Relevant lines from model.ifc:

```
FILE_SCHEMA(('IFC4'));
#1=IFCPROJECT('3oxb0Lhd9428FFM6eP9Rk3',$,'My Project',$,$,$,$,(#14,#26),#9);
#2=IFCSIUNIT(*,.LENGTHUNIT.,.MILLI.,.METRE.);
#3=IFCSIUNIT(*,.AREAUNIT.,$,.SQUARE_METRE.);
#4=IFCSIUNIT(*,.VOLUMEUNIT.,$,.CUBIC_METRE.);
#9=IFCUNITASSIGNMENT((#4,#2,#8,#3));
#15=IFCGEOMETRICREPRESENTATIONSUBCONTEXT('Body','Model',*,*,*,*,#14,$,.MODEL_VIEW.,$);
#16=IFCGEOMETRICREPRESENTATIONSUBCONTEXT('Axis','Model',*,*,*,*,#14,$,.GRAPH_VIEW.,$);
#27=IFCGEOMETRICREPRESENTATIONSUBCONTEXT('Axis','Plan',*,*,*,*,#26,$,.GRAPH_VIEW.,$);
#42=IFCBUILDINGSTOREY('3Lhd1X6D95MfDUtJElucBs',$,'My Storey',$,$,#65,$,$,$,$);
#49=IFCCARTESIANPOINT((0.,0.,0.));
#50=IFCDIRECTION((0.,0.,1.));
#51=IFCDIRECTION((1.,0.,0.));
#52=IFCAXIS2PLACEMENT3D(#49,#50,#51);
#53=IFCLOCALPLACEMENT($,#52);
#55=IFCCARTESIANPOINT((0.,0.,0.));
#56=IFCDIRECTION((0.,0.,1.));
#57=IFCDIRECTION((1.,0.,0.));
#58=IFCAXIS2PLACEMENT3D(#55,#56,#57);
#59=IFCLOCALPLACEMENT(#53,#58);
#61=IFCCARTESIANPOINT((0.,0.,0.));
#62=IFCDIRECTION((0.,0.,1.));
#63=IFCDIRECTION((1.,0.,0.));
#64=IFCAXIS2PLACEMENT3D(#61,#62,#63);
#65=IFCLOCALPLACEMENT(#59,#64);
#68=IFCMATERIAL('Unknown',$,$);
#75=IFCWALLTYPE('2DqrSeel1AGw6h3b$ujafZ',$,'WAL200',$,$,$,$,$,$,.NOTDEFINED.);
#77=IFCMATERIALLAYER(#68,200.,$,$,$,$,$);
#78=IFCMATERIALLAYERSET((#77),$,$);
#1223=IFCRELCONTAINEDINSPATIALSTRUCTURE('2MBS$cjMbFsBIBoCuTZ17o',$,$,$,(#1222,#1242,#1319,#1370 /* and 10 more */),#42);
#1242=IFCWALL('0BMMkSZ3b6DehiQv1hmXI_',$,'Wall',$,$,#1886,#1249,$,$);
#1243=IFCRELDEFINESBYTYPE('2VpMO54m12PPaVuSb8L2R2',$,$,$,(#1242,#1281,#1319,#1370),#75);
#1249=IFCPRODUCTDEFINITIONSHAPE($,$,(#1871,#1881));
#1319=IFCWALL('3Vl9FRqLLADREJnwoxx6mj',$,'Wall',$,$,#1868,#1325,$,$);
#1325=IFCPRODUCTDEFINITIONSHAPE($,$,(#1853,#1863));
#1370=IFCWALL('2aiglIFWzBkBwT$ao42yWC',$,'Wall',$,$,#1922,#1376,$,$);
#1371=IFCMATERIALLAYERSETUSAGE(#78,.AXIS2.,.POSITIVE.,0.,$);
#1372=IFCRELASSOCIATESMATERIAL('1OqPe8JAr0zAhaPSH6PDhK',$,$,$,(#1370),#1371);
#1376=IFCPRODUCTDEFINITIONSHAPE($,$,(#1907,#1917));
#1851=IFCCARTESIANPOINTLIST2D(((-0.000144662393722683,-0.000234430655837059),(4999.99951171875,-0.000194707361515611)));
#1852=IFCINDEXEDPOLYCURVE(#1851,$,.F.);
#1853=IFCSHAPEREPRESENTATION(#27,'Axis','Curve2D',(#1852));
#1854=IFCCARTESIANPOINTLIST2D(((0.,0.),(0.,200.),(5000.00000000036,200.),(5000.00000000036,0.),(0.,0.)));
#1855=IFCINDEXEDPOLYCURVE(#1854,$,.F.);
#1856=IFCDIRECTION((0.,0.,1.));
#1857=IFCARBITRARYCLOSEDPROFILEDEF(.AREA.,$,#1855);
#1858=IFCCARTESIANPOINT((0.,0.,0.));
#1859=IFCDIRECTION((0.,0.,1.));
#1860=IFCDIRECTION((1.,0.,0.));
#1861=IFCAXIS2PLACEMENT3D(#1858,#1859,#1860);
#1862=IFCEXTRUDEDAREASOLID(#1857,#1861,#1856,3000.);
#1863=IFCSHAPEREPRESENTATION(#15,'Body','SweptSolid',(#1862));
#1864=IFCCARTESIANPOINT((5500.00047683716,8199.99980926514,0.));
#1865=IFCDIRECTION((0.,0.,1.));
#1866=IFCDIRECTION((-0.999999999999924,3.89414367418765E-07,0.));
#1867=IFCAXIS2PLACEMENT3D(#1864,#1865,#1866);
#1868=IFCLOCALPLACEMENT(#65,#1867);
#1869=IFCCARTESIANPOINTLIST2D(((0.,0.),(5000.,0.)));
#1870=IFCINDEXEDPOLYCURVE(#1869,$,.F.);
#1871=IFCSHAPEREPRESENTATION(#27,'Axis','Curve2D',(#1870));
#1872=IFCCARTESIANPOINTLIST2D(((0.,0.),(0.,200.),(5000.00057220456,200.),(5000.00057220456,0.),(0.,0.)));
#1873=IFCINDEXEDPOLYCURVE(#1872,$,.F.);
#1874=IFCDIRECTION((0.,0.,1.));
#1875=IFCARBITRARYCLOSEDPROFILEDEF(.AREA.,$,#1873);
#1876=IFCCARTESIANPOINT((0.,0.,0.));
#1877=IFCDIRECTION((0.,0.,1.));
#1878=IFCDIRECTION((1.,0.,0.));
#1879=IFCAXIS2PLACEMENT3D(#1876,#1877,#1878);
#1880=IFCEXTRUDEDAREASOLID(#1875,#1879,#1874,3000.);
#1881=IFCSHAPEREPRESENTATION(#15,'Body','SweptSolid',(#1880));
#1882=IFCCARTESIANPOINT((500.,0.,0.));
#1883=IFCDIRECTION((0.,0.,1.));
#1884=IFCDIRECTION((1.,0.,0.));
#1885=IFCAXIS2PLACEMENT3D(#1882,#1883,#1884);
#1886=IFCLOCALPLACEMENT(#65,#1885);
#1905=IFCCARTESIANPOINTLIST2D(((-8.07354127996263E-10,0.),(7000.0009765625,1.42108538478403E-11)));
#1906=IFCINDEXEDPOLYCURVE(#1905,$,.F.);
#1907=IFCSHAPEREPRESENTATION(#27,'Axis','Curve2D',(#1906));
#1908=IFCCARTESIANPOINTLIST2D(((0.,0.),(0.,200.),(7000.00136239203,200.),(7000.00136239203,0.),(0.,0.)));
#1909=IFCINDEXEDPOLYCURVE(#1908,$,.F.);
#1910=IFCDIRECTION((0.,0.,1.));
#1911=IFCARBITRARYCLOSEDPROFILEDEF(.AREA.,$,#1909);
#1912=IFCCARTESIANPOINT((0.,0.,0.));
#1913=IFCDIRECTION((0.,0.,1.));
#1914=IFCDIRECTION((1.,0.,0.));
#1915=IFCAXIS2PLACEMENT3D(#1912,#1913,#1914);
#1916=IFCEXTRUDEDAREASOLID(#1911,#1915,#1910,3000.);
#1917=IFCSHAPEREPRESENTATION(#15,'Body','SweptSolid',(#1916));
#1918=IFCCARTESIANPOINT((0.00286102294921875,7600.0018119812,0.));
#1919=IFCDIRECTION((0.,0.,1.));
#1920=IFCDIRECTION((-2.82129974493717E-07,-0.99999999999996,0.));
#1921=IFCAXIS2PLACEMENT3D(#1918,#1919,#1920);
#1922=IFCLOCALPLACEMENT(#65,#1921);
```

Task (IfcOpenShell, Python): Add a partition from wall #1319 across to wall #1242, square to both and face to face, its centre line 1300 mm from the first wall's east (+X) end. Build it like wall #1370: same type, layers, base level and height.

```python
import numpy as np
import ifcopenshell
import ifcopenshell.api.geometry
import ifcopenshell.api.material
import ifcopenshell.api.pset
import ifcopenshell.api.root
import ifcopenshell.api.spatial
import ifcopenshell.api.type
import ifcopenshell.geom
import ifcopenshell.util.element
import ifcopenshell.util.placement
import ifcopenshell.util.representation
import ifcopenshell.util.shape
import ifcopenshell.util.unit

model = ifcopenshell.open("model.ifc")
unit_scale = ifcopenshell.util.unit.calculate_unit_scale(model)
settings = ifcopenshell.geom.settings()
settings.set("use-world-coords", True)

start_wall = model.by_id(1319)
end_wall = model.by_guid("0BMMkSZ3b6DehiQv1hmXI_")
like = model.by_id(1370)
matrix = ifcopenshell.util.placement.get_local_placement(start_wall.ObjectPlacement)
matrix[:3, 3] *= unit_scale


def extent(element):
    """Bounding box in the first wall's axes, in metres."""
    shape = ifcopenshell.geom.create_shape(settings, element)
    points = (ifcopenshell.util.shape.get_vertices(shape.geometry) - matrix[:3, 3]) @ matrix[:3, :3]
    return points.min(axis=0), points.max(axis=0)


y_start = extent(start_wall)[1][1]
y_end = extent(end_wall)[0][1]
like_min, like_max = extent(like)
length, height = float(abs(y_end - y_start)), float(like_max[2] - like_min[2])
layer_set = ifcopenshell.util.element.get_material(like, should_skip_usage=True)
thickness = sum(layer.LayerThickness for layer in layer_set.MaterialLayers) * unit_scale

wall = ifcopenshell.api.root.create_entity(model, ifc_class="IfcWall", name="New partition")
storey = ifcopenshell.util.element.get_container(like)
ifcopenshell.api.spatial.assign_container(model, products=[wall], relating_structure=storey)
ifcopenshell.api.type.assign_type(
    model, related_objects=[wall], relating_type=ifcopenshell.util.element.get_type(like), should_map_representations=False
)
rel = ifcopenshell.api.material.assign_material(
    model, products=[wall], type="IfcMaterialLayerSetUsage", material=layer_set
)
rel.RelatingMaterial.OffsetFromReferenceLine = -thickness / 2 / unit_scale
pset = ifcopenshell.api.pset.add_pset(model, product=wall, name="Pset_WallCommon")
ifcopenshell.api.pset.edit_pset(model, pset=pset, properties={"IsExternal": False, "LoadBearing": False})

# The axis runs down the middle of the wall.
axis = ifcopenshell.api.geometry.add_axis_representation(
    model, context=ifcopenshell.util.representation.get_context(model, "Model", "Axis"), axis=[(0.0, 0.0), (length, 0.0)]
)
body = ifcopenshell.api.geometry.add_wall_representation(
    model,
    context=ifcopenshell.util.representation.get_context(model, "Model", "Body", "MODEL_VIEW"),
    length=length,
    height=height,
    thickness=thickness,
    offset=-thickness / 2,
)
for representation in (axis, body):
    ifcopenshell.api.geometry.assign_representation(model, product=wall, representation=representation)

placement = matrix @ ifcopenshell.util.placement.rotation(90, "Z")
placement[:, 3] = matrix @ np.array([extent(start_wall)[0][0] + 1.3, y_start, like_min[2], 1.0])
ifcopenshell.api.geometry.edit_object_placement(model, product=wall, matrix=placement)

print(f"partition {length:.3f} m long, {height:.3f} m high, {thickness:.3f} m thick")

model.write("model_updated.ifc")
```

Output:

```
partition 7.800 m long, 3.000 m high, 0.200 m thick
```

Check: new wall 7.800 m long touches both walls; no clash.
